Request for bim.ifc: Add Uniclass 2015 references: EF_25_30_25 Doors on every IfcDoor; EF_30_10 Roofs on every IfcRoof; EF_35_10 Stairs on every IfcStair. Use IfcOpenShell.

First a look at what the model holds.

```python
import ifcopenshell

model = ifcopenshell.open("bim.ifc")
print(model.schema)
print("classifications:", [c.Name for c in model.by_type("IfcClassification")])
for ifc_class in ("IfcDoor", "IfcRoof", "IfcStair", "IfcWall", "IfcWindow"):
    print(ifc_class, len(model.by_type(ifc_class)))
```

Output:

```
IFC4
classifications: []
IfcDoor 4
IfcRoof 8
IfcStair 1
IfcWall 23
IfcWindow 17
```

```python
import ifcopenshell
import ifcopenshell.api.classification

model = ifcopenshell.open("bim.ifc")

system = ifcopenshell.api.classification.add_classification(model, classification="Uniclass 2015")

codes = {
    "IfcDoor": ("EF_25_30_25", "Doors"),
    "IfcRoof": ("EF_30_10", "Roofs"),
    "IfcStair": ("EF_35_10", "Stairs"),
}
for ifc_class, (code, name) in codes.items():
    products = model.by_type(ifc_class)
    ifcopenshell.api.classification.add_reference(
        model, products=products, classification=system, identification=code, name=name
    )
    print(code, len(products))

model.write("bim-out.ifc")
```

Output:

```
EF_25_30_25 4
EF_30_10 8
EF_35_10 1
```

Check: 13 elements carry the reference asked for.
